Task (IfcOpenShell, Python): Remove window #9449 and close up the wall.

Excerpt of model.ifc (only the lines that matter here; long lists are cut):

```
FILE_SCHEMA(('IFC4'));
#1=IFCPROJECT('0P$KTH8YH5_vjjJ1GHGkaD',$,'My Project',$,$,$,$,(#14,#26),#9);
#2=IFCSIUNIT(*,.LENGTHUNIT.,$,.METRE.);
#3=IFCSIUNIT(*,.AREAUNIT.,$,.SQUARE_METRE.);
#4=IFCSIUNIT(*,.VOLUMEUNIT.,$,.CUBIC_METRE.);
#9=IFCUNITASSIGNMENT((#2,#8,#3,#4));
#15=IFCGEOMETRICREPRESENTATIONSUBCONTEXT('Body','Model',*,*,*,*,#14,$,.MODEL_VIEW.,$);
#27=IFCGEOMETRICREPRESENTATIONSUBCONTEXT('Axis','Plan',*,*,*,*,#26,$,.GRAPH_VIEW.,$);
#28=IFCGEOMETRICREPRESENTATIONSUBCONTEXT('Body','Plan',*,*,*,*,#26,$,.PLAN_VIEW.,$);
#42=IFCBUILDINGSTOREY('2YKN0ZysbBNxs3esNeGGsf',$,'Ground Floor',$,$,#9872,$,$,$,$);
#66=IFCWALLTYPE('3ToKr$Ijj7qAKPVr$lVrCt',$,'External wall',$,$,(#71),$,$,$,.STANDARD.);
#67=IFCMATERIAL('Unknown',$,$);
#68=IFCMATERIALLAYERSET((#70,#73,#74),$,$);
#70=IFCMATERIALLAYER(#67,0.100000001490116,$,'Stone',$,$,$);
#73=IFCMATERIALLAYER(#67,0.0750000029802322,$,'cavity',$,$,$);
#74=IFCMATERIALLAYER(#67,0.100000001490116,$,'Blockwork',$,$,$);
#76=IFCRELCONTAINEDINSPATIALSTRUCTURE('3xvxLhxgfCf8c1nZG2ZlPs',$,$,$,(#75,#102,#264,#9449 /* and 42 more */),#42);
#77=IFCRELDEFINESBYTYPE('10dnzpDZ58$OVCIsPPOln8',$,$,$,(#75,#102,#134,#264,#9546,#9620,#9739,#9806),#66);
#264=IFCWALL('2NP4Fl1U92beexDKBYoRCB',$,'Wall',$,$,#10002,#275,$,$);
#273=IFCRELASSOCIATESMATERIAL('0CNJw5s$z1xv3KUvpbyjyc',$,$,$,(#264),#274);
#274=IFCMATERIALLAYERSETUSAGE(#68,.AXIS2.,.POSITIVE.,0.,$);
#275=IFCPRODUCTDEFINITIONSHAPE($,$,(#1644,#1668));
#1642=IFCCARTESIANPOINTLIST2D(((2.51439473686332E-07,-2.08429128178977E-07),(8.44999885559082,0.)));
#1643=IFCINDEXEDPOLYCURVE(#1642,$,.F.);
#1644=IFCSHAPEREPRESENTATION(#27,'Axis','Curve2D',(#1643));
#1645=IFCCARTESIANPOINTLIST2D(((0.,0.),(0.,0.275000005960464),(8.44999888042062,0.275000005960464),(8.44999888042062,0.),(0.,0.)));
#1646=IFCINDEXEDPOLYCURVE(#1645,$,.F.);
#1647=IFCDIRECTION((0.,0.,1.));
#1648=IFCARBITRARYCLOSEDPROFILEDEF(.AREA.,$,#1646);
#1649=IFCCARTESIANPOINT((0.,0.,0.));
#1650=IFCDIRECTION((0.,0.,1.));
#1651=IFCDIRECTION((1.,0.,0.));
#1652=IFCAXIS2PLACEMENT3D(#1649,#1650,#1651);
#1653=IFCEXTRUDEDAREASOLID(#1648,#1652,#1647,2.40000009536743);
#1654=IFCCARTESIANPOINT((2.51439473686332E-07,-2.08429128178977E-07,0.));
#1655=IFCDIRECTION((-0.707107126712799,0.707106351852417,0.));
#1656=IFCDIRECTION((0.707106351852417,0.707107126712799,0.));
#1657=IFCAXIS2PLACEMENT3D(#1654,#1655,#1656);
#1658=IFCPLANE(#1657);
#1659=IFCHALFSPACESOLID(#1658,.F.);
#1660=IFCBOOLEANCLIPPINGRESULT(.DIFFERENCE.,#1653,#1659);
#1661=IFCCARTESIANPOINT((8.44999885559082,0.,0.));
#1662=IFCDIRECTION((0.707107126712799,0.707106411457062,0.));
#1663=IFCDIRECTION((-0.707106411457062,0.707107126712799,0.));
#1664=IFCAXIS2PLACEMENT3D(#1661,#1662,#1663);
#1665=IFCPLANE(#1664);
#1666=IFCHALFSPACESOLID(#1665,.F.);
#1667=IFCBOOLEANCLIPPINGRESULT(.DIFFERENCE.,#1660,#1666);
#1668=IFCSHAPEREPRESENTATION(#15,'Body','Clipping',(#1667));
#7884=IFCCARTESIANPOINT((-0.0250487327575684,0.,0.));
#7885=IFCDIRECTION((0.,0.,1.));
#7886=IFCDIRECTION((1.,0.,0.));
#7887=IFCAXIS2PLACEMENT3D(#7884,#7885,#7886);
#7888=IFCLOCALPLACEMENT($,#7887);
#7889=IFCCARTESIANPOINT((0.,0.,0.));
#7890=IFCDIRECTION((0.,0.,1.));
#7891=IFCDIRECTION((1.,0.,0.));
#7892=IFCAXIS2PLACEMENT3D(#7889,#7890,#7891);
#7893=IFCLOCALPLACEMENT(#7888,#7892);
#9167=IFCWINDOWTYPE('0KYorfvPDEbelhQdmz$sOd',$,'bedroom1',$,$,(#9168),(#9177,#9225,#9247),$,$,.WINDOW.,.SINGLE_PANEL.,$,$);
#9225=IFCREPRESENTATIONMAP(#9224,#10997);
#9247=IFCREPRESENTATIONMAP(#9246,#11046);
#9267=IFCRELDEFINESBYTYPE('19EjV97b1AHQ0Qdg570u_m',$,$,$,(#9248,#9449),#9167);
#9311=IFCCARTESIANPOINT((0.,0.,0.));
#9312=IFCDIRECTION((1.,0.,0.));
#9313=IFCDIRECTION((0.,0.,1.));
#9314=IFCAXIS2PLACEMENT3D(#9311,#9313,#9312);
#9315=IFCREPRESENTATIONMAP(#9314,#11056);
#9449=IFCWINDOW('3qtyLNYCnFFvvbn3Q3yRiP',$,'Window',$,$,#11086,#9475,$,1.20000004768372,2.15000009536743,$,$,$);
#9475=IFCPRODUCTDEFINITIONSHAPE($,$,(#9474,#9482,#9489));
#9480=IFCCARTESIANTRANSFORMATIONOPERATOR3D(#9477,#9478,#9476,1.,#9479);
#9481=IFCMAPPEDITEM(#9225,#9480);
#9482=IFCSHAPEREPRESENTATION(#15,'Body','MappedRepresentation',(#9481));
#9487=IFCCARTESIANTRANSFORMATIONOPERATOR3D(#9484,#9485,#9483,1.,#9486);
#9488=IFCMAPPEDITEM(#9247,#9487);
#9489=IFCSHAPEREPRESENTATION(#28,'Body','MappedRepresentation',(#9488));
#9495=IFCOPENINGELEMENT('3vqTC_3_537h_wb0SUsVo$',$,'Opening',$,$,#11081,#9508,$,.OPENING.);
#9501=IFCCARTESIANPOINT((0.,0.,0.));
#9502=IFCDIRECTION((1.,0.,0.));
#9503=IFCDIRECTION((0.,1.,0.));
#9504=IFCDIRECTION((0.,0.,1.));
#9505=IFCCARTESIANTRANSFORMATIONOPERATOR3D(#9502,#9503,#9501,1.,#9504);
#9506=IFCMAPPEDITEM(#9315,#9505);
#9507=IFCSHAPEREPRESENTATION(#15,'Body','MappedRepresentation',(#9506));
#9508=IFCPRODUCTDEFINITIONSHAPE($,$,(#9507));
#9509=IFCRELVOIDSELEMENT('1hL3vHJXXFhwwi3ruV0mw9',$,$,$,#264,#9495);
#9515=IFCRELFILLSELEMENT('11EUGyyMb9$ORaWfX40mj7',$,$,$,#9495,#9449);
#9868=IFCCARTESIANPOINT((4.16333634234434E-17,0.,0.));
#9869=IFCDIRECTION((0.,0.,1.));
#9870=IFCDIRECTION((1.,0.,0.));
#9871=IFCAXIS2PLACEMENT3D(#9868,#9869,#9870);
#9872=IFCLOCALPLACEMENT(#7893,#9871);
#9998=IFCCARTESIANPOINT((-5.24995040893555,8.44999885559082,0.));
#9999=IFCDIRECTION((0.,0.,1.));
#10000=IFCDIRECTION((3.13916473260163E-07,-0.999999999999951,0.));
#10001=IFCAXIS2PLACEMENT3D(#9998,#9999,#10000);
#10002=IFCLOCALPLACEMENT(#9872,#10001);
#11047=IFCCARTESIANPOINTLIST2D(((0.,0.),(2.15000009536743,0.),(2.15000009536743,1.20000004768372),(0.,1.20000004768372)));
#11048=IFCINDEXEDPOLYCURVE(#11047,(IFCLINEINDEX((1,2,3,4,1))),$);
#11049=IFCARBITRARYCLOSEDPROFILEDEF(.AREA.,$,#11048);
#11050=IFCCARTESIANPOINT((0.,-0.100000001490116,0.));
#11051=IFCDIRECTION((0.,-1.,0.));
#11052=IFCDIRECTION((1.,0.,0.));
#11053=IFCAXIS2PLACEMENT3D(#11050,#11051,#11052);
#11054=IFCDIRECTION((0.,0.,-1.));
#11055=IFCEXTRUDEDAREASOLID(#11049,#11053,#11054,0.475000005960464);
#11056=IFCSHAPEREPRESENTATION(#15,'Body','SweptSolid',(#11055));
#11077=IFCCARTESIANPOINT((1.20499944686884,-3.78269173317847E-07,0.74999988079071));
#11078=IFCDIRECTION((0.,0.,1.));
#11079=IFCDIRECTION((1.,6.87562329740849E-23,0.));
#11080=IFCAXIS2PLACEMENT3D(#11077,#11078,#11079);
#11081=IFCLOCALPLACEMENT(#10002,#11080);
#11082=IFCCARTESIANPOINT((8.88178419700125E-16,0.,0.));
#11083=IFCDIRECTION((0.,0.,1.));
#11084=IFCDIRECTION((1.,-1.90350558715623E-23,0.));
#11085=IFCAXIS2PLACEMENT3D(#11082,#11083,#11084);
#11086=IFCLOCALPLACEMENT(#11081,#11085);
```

```python
import ifcopenshell
import ifcopenshell.api.feature
import ifcopenshell.api.root
import ifcopenshell.geom
import ifcopenshell.util.shape

model = ifcopenshell.open("model.ifc")
settings = ifcopenshell.geom.settings()


def volume(element):
    """Net volume in cubic metres, openings subtracted."""
    shape = ifcopenshell.geom.create_shape(settings, element)
    return ifcopenshell.util.shape.get_volume(shape.geometry)


window = model.by_guid("3qtyLNYCnFFvvbn3Q3yRiP")
opening = window.FillsVoids[0].RelatingOpeningElement
wall = opening.VoidsElements[0].RelatingBuildingElement
before = volume(wall)

ifcopenshell.api.root.remove_product(model, product=window)
ifcopenshell.api.feature.remove_feature(model, feature=opening)

after = volume(wall)

print(f"wall volume {before:.3f} -> {after:.3f} m3")

model.write("model_updated.ifc")
```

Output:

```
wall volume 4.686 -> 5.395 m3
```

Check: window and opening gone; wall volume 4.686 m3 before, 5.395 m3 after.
